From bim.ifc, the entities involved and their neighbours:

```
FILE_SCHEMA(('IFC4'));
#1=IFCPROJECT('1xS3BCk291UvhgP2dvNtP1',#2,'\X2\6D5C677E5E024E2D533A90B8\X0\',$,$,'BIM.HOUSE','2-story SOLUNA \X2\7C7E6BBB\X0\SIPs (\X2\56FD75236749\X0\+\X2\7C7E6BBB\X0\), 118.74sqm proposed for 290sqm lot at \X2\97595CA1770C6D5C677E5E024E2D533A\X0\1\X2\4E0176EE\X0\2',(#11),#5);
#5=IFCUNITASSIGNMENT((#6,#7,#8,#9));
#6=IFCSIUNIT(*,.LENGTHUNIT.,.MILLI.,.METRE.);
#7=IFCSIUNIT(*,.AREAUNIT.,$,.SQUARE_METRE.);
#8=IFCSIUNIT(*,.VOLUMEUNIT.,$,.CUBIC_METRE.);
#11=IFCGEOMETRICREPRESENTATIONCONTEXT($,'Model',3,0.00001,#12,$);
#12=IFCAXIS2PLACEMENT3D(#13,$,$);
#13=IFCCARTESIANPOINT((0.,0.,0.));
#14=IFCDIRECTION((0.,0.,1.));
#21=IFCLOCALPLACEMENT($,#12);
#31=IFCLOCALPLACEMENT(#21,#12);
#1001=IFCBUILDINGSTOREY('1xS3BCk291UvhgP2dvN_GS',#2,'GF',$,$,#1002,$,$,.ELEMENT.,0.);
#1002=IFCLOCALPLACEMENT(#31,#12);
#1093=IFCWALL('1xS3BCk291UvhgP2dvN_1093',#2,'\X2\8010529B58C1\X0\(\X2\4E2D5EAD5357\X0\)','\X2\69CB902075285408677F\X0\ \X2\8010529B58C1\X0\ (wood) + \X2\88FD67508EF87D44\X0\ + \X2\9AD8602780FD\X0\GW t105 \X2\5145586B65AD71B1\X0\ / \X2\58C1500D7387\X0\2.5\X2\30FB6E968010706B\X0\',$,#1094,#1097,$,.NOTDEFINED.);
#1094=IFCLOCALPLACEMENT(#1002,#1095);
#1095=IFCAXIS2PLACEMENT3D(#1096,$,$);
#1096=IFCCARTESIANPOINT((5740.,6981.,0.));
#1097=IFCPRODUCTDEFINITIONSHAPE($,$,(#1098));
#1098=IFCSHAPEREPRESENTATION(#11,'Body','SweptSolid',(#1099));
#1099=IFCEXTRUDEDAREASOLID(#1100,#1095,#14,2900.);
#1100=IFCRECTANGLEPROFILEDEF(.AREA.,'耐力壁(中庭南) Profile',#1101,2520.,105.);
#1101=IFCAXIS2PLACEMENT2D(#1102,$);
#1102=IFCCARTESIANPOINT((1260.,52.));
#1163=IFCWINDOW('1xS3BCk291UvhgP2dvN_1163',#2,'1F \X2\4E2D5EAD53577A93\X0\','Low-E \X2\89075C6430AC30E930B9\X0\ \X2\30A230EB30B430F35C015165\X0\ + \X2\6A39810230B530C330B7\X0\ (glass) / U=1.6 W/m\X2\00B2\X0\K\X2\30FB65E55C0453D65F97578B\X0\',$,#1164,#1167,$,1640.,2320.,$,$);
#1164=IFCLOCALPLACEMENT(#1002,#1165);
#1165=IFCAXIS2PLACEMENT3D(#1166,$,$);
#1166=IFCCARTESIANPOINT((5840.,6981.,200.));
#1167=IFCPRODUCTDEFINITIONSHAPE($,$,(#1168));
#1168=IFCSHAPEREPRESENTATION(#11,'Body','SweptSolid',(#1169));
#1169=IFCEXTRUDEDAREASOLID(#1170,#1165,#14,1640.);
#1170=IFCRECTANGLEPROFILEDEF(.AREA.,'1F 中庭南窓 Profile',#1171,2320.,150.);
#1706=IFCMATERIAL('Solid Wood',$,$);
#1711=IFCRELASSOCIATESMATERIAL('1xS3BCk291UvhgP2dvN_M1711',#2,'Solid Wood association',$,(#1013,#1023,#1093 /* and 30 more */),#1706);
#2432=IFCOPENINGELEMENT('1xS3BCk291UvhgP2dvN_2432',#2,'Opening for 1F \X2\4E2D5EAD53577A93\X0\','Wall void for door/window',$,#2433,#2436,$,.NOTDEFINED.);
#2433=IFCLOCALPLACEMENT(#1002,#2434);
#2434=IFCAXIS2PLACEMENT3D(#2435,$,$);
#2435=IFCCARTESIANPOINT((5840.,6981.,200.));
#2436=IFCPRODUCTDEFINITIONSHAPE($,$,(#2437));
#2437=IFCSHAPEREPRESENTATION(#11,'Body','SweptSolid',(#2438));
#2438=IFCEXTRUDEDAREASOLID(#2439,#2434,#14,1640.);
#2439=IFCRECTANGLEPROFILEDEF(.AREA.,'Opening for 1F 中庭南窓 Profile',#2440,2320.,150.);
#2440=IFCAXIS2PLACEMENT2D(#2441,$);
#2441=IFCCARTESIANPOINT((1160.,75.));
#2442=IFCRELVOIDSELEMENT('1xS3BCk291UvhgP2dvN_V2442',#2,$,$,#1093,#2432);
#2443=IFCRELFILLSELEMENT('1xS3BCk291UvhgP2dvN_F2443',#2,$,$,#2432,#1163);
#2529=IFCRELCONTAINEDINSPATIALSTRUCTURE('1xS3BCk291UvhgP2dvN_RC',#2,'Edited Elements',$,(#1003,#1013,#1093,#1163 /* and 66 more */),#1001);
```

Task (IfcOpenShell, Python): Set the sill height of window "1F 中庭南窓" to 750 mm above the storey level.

```python
import numpy as np
import ifcopenshell
import ifcopenshell.api.geometry
import ifcopenshell.geom
import ifcopenshell.util.element
import ifcopenshell.util.placement
import ifcopenshell.util.shape
import ifcopenshell.util.unit

model = ifcopenshell.open("bim.ifc")
unit_scale = ifcopenshell.util.unit.calculate_unit_scale(model)

window = model.by_guid("1xS3BCk291UvhgP2dvN_1163")
opening = window.FillsVoids[0].RelatingOpeningElement
storey = ifcopenshell.util.element.get_container(window, ifc_class="IfcBuildingStorey")
level = ifcopenshell.util.placement.get_local_placement(storey.ObjectPlacement)[2, 3]

# The opening's origin need not be at the sill, so measure its lowest point.
shape = ifcopenshell.geom.create_shape(ifcopenshell.geom.settings(), opening)
bottom = ifcopenshell.util.shape.get_shape_bottom_elevation(shape, shape.geometry) / unit_scale
dz = level + 0.75 / unit_scale - bottom

shift = np.array([0.0, 0.0, dz])
# The window is not placed relative to its opening, so move both.
for product in (opening, window):
    matrix = ifcopenshell.util.placement.get_local_placement(product.ObjectPlacement)
    matrix[:3, 3] += shift
    ifcopenshell.api.geometry.edit_object_placement(model, product=product, matrix=matrix, is_si=False)

print(f"moved by {dz * unit_scale:+.3f} m")

model.write("bim_updated.ifc")
```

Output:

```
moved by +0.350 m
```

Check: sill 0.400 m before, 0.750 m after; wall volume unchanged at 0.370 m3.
